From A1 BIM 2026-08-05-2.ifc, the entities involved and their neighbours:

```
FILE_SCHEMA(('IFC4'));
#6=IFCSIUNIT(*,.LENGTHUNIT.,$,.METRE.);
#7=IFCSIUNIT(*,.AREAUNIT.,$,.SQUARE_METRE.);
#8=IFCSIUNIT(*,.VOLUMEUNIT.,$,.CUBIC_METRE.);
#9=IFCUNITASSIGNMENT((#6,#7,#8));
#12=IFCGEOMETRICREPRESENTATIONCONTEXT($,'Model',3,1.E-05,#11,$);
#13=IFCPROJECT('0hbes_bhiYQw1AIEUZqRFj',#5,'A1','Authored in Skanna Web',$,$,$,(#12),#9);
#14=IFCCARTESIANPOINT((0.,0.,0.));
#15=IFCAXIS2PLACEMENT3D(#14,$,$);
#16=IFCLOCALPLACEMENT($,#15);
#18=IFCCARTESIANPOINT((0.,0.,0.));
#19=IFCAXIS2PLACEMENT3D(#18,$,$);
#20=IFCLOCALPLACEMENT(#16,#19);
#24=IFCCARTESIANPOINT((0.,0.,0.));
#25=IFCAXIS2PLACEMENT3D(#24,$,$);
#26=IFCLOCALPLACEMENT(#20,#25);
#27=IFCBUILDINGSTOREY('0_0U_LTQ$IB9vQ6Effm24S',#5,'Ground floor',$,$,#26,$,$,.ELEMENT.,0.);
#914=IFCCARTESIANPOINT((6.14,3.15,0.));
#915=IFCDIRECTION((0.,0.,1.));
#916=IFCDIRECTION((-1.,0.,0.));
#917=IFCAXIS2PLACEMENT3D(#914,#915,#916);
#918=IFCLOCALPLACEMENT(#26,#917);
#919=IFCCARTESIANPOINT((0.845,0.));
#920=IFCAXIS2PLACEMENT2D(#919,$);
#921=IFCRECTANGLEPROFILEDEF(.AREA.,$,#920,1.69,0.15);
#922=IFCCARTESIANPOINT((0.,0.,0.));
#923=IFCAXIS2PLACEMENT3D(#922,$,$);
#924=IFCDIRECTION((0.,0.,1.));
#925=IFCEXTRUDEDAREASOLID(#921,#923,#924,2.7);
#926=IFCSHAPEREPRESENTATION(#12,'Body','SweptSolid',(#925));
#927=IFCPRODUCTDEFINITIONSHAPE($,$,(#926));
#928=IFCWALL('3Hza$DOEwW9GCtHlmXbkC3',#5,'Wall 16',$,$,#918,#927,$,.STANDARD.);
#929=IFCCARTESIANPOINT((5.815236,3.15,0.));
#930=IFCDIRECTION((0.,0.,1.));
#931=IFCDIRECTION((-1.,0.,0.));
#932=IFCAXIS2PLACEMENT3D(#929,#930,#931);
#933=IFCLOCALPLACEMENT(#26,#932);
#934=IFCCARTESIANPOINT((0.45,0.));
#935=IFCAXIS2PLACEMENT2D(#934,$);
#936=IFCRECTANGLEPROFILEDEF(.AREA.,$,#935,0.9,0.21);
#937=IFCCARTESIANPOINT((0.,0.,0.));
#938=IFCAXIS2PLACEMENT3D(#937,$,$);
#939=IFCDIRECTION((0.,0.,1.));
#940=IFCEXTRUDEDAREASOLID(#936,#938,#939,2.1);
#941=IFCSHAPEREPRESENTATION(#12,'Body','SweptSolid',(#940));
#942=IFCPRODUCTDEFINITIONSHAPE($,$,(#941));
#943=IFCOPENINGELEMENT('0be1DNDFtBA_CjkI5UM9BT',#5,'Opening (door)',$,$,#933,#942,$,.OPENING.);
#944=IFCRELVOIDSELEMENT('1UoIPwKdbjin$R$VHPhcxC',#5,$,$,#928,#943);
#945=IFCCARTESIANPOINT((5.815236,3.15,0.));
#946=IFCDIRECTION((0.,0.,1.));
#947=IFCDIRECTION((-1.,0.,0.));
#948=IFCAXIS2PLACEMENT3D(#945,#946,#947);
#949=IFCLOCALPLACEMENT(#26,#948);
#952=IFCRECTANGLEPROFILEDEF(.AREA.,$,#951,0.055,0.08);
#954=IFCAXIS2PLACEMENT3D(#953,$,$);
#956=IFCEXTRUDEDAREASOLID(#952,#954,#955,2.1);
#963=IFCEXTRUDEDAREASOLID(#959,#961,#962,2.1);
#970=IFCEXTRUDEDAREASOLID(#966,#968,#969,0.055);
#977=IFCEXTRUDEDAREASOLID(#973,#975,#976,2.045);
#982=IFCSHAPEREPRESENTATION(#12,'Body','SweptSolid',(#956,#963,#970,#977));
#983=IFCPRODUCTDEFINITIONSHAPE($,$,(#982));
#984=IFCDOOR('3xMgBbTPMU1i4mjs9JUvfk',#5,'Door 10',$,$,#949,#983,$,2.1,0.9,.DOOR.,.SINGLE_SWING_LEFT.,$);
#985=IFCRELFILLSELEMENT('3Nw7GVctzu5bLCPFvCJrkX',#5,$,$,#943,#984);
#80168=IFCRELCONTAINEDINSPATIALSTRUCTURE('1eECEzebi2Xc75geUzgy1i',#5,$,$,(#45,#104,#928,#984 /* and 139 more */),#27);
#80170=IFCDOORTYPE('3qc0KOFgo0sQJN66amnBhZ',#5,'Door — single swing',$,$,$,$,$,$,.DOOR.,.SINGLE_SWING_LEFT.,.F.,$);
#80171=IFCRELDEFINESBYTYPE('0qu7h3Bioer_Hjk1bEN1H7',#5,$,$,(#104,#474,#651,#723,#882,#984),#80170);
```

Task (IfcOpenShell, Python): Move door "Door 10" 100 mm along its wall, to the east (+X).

```python
import ifcopenshell
import ifcopenshell.api.geometry
import ifcopenshell.util.placement
import ifcopenshell.util.unit

model = ifcopenshell.open("A1 BIM 2026-08-05-2.ifc")
unit_scale = ifcopenshell.util.unit.calculate_unit_scale(model)

door = model.by_guid("3xMgBbTPMU1i4mjs9JUvfk")
opening = door.FillsVoids[0].RelatingOpeningElement
wall = opening.VoidsElements[0].RelatingBuildingElement

wall_matrix = ifcopenshell.util.placement.get_local_placement(wall.ObjectPlacement)
shift = wall_matrix[:3, 0] * -0.1 / unit_scale
before = ifcopenshell.util.placement.get_local_placement(door.ObjectPlacement)[:3, 3].copy()

# The door is not placed relative to its opening, so move both.
for product in (opening, door):
    matrix = ifcopenshell.util.placement.get_local_placement(product.ObjectPlacement)
    matrix[:3, 3] += shift
    ifcopenshell.api.geometry.edit_object_placement(model, product=product, matrix=matrix, is_si=False)

after = ifcopenshell.util.placement.get_local_placement(door.ObjectPlacement)[:3, 3]
print("door moved by", (after - before).round(3) + 0.0)

model.write("A1 BIM 2026-08-05-2_rev.ifc")
```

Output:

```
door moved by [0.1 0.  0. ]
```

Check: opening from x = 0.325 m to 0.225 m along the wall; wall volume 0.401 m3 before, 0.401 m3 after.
